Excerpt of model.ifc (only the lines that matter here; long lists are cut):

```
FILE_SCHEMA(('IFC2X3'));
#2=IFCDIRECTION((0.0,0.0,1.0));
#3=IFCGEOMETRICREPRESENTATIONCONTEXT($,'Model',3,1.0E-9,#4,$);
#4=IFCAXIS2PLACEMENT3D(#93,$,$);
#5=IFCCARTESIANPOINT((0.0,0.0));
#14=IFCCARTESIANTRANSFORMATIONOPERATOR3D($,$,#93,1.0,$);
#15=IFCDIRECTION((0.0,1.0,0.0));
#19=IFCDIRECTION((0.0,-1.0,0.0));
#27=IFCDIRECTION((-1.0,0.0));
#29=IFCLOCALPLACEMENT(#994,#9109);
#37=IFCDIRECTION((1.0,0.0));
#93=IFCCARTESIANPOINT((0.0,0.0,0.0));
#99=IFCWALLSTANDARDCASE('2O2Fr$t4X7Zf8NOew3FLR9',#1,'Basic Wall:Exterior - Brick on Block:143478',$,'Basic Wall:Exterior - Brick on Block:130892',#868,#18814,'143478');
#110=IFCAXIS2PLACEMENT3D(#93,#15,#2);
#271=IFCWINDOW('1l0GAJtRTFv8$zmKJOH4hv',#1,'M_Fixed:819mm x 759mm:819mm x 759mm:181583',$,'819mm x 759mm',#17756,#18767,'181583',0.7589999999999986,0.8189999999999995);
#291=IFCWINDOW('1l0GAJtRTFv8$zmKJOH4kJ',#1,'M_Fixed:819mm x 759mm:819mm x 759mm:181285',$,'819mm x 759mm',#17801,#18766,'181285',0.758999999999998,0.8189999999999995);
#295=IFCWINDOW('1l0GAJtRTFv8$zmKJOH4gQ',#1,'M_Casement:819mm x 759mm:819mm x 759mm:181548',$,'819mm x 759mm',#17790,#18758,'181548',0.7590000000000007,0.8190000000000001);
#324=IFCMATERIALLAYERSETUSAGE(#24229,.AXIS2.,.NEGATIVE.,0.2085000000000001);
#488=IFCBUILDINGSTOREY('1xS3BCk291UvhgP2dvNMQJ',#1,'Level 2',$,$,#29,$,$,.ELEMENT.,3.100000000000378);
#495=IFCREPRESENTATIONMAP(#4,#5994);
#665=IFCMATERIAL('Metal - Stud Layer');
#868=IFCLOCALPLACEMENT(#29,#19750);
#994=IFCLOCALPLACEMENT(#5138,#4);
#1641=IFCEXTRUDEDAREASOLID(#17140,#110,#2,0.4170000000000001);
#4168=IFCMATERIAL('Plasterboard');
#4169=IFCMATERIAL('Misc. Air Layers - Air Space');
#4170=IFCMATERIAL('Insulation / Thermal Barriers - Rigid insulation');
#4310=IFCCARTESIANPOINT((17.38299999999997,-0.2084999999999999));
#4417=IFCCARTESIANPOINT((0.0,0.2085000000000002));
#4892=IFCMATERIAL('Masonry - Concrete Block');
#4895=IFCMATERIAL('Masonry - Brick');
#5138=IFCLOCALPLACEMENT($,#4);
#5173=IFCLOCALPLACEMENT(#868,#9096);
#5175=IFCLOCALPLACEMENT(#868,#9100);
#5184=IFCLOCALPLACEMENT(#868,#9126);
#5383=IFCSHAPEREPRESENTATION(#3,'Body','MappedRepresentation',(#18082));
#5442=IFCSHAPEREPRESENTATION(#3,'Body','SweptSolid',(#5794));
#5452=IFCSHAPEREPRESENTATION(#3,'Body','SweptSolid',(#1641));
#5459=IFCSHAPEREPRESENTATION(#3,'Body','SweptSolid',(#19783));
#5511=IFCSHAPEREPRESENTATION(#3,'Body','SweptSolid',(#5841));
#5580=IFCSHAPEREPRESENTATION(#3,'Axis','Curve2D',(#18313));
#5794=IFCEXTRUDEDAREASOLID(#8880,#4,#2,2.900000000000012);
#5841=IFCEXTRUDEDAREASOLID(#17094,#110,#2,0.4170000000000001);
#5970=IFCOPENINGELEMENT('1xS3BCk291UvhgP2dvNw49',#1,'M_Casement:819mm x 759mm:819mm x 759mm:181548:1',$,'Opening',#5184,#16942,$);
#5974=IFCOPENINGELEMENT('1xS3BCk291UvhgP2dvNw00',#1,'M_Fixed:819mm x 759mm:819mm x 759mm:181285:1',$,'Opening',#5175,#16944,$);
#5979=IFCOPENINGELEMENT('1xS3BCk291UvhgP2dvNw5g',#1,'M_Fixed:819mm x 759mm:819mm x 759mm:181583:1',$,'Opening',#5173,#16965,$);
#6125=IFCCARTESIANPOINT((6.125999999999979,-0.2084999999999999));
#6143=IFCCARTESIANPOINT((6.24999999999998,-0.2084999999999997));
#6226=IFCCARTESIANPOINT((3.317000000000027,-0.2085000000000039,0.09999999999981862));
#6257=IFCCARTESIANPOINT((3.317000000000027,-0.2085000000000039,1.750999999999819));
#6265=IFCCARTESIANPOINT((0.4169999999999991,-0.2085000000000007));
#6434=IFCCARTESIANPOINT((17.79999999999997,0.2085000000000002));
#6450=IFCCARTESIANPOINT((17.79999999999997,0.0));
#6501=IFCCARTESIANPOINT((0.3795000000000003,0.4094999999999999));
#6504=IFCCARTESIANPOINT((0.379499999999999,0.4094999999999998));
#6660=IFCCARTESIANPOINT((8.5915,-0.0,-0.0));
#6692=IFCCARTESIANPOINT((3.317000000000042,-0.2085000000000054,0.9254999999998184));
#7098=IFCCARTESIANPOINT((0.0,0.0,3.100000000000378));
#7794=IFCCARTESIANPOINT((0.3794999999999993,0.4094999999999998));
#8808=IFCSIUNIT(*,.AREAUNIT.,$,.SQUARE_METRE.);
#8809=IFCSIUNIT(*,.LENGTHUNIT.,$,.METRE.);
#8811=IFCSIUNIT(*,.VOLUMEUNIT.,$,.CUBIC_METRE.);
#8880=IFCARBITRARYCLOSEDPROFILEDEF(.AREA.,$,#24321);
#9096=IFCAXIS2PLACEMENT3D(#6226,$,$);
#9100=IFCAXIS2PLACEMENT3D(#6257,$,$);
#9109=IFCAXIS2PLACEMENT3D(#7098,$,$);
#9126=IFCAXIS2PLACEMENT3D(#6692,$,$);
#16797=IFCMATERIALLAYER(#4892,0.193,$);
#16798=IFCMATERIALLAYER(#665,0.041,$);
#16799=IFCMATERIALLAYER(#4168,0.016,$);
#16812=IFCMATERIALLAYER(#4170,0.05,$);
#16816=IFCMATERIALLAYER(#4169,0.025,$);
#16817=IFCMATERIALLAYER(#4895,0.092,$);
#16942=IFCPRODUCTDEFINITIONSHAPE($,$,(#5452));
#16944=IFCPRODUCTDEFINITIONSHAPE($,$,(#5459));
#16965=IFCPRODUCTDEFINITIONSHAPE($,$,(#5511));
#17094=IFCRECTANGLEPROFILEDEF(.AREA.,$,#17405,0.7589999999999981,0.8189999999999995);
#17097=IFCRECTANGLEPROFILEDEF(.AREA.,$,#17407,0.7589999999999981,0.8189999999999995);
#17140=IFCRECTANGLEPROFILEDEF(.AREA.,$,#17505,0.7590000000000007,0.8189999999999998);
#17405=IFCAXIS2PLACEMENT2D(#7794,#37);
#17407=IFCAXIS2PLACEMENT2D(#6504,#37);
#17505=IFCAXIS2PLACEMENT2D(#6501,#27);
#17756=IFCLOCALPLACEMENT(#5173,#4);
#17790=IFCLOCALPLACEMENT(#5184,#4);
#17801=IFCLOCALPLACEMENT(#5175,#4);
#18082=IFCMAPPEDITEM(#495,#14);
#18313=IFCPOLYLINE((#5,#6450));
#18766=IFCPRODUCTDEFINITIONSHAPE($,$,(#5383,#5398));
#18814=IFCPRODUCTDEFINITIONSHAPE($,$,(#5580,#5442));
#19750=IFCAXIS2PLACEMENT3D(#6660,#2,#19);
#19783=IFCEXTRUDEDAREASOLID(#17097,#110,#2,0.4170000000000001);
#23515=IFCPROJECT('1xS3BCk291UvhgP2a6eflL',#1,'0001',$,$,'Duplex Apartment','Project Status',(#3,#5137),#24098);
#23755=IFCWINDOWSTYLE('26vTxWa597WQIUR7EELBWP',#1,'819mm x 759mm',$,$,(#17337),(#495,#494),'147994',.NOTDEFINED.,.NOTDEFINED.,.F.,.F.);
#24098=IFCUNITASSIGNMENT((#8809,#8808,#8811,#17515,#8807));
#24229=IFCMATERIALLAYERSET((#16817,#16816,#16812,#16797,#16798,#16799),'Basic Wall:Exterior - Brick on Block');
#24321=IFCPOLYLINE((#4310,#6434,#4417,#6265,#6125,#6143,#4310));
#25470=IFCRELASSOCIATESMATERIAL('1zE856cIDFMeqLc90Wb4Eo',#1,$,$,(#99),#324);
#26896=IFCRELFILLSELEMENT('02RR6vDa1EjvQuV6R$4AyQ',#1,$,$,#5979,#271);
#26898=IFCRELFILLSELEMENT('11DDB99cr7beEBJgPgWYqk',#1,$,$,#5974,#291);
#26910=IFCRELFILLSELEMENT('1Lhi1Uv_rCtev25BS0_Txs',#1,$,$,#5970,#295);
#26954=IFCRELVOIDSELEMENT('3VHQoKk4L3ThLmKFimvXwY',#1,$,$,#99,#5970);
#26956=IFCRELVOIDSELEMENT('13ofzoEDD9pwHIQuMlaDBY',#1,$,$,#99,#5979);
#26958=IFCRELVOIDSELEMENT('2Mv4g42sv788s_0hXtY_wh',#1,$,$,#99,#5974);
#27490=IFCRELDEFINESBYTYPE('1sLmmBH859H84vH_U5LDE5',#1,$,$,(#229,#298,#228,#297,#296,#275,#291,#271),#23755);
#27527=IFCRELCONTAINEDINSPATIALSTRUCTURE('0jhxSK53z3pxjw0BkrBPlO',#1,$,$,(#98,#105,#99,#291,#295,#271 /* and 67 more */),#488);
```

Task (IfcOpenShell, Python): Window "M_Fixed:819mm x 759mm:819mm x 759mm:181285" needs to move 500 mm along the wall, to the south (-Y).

```python
import ifcopenshell
import ifcopenshell.api.geometry
import ifcopenshell.util.placement
import ifcopenshell.util.unit

model = ifcopenshell.open("model.ifc")
unit_scale = ifcopenshell.util.unit.calculate_unit_scale(model)

window = model.by_guid("1l0GAJtRTFv8$zmKJOH4kJ")
opening = window.FillsVoids[0].RelatingOpeningElement
wall = opening.VoidsElements[0].RelatingBuildingElement

wall_matrix = ifcopenshell.util.placement.get_local_placement(wall.ObjectPlacement)
shift = wall_matrix[:3, 0] * 0.5 / unit_scale
before = ifcopenshell.util.placement.get_local_placement(window.ObjectPlacement)[:3, 3].copy()

# The window is placed relative to its opening, so it follows when the opening moves.
matrix = ifcopenshell.util.placement.get_local_placement(opening.ObjectPlacement)
matrix[:3, 3] += shift
ifcopenshell.api.geometry.edit_object_placement(
    model, product=opening, matrix=matrix, is_si=False, should_transform_children=True
)

after = ifcopenshell.util.placement.get_local_placement(window.ObjectPlacement)[:3, 3]
print("window moved by", (after - before).round(3) + 0.0)

model.write("model_rev.ifc")
```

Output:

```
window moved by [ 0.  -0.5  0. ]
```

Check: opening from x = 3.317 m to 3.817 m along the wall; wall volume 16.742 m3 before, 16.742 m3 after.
